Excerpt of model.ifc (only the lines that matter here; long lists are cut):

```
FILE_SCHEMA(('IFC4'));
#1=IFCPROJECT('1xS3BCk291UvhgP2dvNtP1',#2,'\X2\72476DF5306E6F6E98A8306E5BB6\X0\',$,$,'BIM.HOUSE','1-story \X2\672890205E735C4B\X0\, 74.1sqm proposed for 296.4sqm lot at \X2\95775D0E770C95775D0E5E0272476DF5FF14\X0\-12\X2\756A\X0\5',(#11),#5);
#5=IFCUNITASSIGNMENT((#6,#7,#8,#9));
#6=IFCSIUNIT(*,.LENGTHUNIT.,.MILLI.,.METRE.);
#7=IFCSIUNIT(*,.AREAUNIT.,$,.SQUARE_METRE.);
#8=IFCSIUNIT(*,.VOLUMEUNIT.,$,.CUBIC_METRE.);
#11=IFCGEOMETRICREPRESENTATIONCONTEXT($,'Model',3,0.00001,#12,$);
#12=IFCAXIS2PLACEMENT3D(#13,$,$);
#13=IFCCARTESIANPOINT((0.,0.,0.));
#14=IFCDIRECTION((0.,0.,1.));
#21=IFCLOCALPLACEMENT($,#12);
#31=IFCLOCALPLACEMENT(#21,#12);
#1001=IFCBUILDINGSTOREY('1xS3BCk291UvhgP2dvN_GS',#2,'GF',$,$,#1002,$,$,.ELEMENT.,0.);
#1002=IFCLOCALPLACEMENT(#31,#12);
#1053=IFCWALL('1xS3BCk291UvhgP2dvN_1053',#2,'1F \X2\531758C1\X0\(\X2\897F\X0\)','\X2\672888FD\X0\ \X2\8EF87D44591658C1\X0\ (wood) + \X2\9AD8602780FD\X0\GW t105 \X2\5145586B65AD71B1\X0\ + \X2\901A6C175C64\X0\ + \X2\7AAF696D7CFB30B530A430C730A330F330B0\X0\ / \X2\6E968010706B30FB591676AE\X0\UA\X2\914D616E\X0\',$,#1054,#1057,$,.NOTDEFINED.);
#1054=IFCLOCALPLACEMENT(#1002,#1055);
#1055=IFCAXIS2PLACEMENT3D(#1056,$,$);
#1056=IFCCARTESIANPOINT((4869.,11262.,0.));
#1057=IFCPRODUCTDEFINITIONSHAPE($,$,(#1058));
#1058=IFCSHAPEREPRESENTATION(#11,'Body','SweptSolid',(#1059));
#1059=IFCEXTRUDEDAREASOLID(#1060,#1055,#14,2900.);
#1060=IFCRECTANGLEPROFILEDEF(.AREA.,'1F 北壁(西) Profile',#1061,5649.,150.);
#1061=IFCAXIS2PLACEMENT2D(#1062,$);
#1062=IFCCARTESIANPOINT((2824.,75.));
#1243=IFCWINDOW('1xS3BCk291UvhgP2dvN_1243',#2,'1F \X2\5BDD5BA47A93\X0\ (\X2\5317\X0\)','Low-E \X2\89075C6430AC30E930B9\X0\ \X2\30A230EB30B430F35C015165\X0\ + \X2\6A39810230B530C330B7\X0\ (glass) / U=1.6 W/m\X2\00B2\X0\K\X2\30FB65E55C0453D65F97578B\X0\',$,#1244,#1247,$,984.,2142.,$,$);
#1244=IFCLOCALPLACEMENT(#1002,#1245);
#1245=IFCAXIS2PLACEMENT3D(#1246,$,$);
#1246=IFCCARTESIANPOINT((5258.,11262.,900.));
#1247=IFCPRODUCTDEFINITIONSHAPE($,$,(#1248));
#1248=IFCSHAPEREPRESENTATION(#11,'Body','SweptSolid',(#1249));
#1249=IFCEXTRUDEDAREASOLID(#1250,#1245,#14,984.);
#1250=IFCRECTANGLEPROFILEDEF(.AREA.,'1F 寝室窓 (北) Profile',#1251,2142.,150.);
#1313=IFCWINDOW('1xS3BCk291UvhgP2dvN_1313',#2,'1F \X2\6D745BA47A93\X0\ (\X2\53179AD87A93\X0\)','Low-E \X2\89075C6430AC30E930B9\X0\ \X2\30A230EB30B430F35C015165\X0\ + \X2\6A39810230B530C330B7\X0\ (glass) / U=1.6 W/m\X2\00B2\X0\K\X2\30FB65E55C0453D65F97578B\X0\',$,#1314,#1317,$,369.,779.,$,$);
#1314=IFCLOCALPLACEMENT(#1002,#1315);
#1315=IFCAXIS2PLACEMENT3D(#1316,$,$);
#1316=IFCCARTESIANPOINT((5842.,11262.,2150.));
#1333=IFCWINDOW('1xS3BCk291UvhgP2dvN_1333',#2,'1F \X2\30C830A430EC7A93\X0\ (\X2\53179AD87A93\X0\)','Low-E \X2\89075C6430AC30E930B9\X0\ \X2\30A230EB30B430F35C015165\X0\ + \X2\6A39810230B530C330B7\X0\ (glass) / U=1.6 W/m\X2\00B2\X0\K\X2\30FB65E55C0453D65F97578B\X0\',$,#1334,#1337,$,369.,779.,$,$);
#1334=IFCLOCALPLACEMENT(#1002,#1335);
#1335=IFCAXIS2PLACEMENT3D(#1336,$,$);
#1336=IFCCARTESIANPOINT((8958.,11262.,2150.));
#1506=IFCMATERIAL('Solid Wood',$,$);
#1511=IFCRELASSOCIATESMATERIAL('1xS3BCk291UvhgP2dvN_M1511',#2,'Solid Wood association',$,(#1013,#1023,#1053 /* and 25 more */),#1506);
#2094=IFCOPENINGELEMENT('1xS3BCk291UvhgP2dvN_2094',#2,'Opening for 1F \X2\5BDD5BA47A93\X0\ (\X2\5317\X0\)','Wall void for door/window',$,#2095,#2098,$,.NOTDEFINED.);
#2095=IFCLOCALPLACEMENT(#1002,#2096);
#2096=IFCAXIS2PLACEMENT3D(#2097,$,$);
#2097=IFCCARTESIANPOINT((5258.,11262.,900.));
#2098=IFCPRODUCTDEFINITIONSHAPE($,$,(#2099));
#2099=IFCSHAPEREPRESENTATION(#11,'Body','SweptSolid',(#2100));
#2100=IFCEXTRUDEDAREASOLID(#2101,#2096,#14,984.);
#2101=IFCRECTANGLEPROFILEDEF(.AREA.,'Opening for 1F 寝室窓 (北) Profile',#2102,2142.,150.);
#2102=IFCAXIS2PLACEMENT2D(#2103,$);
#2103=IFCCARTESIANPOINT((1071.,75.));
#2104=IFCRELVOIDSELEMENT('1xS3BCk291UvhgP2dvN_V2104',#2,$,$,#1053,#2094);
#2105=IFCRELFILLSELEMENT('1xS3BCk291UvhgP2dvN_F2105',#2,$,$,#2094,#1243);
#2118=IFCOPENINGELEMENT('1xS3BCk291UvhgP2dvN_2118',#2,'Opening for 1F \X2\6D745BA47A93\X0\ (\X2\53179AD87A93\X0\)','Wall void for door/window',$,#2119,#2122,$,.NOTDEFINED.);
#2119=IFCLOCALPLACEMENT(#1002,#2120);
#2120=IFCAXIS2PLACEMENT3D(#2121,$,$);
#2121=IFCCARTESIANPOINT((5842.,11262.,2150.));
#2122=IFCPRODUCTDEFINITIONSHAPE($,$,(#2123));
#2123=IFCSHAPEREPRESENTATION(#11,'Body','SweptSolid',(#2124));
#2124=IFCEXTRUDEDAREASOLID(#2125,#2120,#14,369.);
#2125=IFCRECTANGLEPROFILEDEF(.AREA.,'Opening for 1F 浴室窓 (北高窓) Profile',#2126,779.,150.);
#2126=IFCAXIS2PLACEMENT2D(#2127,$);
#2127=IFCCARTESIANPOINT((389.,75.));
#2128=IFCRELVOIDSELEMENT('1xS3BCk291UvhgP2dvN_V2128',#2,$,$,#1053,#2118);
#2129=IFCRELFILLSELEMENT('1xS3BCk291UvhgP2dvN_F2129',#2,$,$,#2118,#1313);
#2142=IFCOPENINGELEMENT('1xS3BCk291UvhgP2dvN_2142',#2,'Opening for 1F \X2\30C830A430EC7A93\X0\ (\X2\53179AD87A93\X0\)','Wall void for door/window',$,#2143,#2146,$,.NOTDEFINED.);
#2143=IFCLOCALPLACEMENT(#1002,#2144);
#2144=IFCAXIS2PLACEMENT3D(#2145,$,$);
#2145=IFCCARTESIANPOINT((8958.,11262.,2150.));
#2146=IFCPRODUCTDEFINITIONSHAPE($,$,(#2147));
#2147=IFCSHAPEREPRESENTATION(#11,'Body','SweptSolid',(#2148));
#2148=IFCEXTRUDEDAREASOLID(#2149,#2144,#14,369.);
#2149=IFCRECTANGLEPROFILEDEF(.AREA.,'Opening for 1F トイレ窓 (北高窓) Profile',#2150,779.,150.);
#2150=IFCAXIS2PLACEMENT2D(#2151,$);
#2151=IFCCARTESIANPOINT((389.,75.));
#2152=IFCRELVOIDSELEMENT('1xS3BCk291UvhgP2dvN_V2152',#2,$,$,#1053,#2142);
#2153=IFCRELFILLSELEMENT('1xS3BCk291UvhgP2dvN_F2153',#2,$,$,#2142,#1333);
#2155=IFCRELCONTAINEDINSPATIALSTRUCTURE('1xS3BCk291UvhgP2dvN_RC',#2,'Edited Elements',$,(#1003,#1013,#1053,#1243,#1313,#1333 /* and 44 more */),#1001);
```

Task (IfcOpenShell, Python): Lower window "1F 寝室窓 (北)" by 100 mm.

```python
import numpy as np
import ifcopenshell
import ifcopenshell.api.geometry
import ifcopenshell.util.placement
import ifcopenshell.util.unit

model = ifcopenshell.open("model.ifc")
unit_scale = ifcopenshell.util.unit.calculate_unit_scale(model)

window = model.by_guid("1xS3BCk291UvhgP2dvN_1243")
opening = window.FillsVoids[0].RelatingOpeningElement
dz = -0.1 / unit_scale

shift = np.array([0.0, 0.0, dz])
# The window is not placed relative to its opening, so move both.
for product in (opening, window):
    matrix = ifcopenshell.util.placement.get_local_placement(product.ObjectPlacement)
    matrix[:3, 3] += shift
    ifcopenshell.api.geometry.edit_object_placement(model, product=product, matrix=matrix, is_si=False)

print(f"moved by {dz * unit_scale:+.3f} m")

model.write("model_updated.ifc")
```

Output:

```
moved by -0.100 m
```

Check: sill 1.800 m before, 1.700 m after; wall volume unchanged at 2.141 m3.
